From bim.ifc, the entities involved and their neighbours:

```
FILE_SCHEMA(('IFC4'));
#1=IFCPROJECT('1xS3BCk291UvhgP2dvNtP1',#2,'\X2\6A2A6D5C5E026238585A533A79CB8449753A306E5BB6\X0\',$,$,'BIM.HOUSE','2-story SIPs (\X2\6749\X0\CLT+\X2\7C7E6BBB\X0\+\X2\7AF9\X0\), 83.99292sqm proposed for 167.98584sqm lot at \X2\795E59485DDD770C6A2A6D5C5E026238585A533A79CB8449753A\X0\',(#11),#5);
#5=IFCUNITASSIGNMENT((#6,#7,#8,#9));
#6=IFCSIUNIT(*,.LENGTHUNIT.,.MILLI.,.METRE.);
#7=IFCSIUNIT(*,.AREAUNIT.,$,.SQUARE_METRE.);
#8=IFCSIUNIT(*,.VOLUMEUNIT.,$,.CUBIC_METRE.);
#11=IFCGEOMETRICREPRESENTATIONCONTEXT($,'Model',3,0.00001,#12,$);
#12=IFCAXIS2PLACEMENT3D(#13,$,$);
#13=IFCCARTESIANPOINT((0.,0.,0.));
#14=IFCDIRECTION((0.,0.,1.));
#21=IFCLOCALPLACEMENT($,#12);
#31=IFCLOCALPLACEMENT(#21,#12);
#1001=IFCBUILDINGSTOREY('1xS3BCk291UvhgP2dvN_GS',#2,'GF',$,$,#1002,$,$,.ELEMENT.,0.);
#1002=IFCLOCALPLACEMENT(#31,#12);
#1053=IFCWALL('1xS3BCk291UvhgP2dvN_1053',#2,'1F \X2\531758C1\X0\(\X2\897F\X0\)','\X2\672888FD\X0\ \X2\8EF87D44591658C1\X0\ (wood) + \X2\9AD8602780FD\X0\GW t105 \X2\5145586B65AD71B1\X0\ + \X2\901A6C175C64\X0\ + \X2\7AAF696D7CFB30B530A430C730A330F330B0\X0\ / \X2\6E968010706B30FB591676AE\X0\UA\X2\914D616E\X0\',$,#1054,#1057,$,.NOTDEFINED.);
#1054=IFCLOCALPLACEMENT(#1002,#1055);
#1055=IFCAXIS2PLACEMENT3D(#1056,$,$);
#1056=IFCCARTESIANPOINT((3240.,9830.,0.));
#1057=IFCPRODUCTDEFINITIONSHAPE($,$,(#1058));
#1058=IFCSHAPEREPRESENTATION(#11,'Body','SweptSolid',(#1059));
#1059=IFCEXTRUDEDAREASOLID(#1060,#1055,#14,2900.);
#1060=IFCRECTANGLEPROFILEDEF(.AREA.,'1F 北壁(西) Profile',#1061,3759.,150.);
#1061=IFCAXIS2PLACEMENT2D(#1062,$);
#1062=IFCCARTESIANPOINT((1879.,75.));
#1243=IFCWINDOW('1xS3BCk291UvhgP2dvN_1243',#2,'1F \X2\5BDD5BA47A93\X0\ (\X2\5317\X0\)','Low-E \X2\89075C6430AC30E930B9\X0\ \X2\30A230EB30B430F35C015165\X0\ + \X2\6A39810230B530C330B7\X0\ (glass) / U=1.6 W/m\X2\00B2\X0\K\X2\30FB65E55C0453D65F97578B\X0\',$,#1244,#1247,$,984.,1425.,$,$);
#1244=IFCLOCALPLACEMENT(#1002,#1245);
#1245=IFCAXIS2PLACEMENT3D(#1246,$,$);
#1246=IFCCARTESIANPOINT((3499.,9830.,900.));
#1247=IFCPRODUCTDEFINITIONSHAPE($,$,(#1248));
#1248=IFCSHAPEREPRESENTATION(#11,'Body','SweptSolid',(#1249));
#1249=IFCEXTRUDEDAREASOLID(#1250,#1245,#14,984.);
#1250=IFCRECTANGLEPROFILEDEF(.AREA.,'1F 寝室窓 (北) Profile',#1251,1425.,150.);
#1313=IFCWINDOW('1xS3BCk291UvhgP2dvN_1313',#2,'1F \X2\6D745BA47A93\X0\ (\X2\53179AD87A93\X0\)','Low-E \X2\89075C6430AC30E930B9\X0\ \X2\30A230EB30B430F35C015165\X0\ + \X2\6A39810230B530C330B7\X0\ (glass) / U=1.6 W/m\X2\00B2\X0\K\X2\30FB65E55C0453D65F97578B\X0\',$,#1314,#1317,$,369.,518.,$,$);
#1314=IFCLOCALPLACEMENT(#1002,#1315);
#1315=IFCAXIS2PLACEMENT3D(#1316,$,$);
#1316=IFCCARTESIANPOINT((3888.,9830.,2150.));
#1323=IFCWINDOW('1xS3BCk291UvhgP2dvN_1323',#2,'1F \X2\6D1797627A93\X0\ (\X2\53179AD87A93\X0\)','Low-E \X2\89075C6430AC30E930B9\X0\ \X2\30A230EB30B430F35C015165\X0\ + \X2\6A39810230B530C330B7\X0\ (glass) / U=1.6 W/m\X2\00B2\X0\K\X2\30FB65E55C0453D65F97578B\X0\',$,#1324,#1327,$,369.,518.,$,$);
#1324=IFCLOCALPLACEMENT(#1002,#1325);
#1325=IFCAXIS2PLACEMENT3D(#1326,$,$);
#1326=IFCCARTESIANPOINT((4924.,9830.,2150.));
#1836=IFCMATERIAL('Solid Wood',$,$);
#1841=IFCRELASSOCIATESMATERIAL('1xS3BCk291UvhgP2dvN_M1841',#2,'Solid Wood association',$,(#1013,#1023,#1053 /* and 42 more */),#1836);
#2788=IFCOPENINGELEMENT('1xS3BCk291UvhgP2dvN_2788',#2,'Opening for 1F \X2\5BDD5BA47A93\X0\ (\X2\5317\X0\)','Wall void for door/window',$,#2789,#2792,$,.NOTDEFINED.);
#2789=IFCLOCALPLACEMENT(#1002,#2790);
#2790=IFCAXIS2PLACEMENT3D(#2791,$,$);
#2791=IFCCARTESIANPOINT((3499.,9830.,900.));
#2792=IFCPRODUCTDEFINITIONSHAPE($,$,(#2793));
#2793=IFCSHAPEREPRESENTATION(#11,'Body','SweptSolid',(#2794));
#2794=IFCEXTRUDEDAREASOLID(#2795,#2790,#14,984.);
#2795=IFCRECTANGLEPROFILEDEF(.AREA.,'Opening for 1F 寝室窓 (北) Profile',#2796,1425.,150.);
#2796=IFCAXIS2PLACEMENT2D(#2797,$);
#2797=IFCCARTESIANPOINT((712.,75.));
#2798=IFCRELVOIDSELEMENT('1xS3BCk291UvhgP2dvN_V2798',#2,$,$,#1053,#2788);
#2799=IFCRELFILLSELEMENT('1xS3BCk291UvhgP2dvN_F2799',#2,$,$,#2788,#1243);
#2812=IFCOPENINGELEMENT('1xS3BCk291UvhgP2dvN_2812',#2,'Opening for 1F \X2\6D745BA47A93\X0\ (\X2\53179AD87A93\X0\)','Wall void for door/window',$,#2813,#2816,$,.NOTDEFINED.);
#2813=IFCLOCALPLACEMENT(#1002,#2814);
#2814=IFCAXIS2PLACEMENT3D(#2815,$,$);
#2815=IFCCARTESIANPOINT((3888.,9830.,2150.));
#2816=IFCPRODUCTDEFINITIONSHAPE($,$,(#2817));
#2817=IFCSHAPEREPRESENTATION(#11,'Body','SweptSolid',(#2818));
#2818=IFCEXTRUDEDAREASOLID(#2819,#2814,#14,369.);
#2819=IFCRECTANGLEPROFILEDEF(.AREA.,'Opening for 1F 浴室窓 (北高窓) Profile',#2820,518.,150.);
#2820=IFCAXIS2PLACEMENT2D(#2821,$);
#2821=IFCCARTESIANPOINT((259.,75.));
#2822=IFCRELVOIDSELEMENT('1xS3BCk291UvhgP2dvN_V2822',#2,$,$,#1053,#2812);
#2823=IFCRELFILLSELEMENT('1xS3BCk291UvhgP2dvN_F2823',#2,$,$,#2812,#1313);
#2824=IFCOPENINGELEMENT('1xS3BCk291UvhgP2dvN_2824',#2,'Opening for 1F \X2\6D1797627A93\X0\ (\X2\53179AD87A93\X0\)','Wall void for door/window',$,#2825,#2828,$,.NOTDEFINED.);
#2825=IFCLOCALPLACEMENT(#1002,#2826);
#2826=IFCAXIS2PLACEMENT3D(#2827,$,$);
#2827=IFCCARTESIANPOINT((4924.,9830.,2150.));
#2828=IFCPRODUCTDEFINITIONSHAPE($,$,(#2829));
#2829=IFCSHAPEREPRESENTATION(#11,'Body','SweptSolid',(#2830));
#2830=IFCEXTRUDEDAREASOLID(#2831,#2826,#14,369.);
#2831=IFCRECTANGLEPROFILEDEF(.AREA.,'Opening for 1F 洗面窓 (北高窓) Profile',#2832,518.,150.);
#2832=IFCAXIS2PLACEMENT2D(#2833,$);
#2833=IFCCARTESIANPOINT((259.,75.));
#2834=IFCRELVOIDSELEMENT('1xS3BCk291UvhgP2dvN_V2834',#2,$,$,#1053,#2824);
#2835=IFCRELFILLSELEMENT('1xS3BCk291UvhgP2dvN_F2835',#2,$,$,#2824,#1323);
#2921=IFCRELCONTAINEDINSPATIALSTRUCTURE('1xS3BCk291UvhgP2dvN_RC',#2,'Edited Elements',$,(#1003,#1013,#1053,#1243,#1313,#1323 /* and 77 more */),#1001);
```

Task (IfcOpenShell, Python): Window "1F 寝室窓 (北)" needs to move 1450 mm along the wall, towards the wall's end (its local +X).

```python
import ifcopenshell
import ifcopenshell.api.geometry
import ifcopenshell.util.placement

model = ifcopenshell.open("bim.ifc")

window = model.by_guid("1xS3BCk291UvhgP2dvN_1243")
opening = window.FillsVoids[0].RelatingOpeningElement
wall = opening.VoidsElements[0].RelatingBuildingElement

wall_matrix = ifcopenshell.util.placement.get_local_placement(wall.ObjectPlacement)
shift = wall_matrix[:3, 0] * 1450.0
before = ifcopenshell.util.placement.get_local_placement(window.ObjectPlacement)[:3, 3].copy()

# The window is not placed relative to its opening, so move both.
for product in (opening, window):
    matrix = ifcopenshell.util.placement.get_local_placement(product.ObjectPlacement)
    matrix[:3, 3] += shift
    ifcopenshell.api.geometry.edit_object_placement(model, product=product, matrix=matrix, is_si=False)

after = ifcopenshell.util.placement.get_local_placement(window.ObjectPlacement)[:3, 3]
print("window moved by", (after - before).round(3) + 0.0)

model.write("bim_updated.ifc")
```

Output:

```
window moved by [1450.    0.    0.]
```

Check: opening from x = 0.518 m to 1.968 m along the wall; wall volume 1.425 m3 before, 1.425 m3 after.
